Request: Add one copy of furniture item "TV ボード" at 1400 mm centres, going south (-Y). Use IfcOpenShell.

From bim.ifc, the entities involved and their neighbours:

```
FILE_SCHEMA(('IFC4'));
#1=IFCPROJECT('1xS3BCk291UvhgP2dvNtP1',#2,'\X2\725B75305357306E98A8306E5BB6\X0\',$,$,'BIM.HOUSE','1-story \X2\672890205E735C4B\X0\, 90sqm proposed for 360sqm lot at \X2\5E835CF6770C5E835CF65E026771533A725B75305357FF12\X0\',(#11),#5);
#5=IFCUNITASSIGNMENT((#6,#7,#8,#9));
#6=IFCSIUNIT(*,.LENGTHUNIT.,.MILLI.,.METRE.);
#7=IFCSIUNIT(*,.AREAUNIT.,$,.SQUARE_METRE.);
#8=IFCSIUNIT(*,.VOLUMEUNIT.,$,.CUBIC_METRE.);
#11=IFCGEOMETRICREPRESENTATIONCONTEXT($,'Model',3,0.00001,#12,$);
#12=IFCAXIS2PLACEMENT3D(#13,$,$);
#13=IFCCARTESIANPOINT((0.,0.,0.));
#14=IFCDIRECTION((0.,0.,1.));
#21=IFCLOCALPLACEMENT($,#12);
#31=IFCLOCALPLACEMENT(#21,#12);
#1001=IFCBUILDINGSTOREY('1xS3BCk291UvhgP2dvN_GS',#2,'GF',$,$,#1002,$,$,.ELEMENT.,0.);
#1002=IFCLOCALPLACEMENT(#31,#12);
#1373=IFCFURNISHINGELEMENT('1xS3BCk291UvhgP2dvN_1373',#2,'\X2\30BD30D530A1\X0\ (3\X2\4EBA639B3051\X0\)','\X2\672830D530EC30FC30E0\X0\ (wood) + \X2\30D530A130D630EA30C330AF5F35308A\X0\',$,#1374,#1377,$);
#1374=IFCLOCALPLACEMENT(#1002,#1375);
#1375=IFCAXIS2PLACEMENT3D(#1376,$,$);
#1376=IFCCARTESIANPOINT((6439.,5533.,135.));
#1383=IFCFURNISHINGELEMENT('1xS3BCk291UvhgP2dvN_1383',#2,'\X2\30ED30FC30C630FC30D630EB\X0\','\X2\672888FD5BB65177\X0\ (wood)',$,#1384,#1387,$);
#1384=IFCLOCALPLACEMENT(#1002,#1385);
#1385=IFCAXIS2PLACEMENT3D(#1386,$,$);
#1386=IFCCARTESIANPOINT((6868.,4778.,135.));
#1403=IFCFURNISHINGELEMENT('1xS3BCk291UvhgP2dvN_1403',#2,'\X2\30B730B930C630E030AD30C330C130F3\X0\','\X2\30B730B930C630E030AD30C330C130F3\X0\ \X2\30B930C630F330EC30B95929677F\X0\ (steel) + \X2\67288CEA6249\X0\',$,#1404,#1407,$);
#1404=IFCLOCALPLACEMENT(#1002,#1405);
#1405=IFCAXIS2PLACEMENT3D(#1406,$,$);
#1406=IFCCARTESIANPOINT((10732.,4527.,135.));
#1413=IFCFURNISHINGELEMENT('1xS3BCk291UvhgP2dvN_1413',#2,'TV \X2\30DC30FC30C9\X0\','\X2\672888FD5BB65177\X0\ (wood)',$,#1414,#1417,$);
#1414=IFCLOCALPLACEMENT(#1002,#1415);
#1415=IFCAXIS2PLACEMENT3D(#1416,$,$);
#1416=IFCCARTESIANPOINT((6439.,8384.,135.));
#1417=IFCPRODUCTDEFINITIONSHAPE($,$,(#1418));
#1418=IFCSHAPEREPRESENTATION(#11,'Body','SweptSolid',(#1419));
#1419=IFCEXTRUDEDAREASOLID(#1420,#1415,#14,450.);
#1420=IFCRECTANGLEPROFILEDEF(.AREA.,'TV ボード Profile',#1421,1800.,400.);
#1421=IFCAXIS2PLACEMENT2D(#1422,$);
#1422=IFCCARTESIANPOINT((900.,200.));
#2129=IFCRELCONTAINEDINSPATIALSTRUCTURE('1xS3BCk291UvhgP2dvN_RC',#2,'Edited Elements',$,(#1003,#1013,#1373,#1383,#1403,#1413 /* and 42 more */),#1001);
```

```python
import numpy as np
import ifcopenshell
import ifcopenshell.api.geometry
import ifcopenshell.api.root
import ifcopenshell.util.element
import ifcopenshell.util.placement
import ifcopenshell.util.unit

model = ifcopenshell.open("bim.ifc")
unit_scale = ifcopenshell.util.unit.calculate_unit_scale(model)


def reuse_history(source, copy):
    """copy_class also copies each property set's owner history, people and application; keep the originals."""
    for rel in copy.IsDefinedBy:
        if rel.is_a("IfcRelDefinesByProperties") and (history := rel.RelatingPropertyDefinition.OwnerHistory):
            rel.RelatingPropertyDefinition.OwnerHistory = source.OwnerHistory
            ifcopenshell.util.element.remove_deep2(model, history)


source = model.by_guid("1xS3BCk291UvhgP2dvN_1413")
base = ifcopenshell.util.placement.get_local_placement(source.ObjectPlacement)
step = np.array([0.0, -1.0, 0.0]) * 1.4 / unit_scale

for i in range(1, 2):
    copy = ifcopenshell.api.root.copy_class(model, product=source)
    copy.Representation = ifcopenshell.util.element.copy_deep(
        model, source.Representation, exclude=["IfcGeometricRepresentationContext", "IfcRepresentationMap"]
    )
    reuse_history(source, copy)
    matrix = base.copy()
    matrix[:3, 3] += i * step
    print("added at", matrix[:3, 3].round(3) + 0.0)
    ifcopenshell.api.geometry.edit_object_placement(model, product=copy, matrix=matrix, is_si=False)

model.write("bim_updated.ifc")
```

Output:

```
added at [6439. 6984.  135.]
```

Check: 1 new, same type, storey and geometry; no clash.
